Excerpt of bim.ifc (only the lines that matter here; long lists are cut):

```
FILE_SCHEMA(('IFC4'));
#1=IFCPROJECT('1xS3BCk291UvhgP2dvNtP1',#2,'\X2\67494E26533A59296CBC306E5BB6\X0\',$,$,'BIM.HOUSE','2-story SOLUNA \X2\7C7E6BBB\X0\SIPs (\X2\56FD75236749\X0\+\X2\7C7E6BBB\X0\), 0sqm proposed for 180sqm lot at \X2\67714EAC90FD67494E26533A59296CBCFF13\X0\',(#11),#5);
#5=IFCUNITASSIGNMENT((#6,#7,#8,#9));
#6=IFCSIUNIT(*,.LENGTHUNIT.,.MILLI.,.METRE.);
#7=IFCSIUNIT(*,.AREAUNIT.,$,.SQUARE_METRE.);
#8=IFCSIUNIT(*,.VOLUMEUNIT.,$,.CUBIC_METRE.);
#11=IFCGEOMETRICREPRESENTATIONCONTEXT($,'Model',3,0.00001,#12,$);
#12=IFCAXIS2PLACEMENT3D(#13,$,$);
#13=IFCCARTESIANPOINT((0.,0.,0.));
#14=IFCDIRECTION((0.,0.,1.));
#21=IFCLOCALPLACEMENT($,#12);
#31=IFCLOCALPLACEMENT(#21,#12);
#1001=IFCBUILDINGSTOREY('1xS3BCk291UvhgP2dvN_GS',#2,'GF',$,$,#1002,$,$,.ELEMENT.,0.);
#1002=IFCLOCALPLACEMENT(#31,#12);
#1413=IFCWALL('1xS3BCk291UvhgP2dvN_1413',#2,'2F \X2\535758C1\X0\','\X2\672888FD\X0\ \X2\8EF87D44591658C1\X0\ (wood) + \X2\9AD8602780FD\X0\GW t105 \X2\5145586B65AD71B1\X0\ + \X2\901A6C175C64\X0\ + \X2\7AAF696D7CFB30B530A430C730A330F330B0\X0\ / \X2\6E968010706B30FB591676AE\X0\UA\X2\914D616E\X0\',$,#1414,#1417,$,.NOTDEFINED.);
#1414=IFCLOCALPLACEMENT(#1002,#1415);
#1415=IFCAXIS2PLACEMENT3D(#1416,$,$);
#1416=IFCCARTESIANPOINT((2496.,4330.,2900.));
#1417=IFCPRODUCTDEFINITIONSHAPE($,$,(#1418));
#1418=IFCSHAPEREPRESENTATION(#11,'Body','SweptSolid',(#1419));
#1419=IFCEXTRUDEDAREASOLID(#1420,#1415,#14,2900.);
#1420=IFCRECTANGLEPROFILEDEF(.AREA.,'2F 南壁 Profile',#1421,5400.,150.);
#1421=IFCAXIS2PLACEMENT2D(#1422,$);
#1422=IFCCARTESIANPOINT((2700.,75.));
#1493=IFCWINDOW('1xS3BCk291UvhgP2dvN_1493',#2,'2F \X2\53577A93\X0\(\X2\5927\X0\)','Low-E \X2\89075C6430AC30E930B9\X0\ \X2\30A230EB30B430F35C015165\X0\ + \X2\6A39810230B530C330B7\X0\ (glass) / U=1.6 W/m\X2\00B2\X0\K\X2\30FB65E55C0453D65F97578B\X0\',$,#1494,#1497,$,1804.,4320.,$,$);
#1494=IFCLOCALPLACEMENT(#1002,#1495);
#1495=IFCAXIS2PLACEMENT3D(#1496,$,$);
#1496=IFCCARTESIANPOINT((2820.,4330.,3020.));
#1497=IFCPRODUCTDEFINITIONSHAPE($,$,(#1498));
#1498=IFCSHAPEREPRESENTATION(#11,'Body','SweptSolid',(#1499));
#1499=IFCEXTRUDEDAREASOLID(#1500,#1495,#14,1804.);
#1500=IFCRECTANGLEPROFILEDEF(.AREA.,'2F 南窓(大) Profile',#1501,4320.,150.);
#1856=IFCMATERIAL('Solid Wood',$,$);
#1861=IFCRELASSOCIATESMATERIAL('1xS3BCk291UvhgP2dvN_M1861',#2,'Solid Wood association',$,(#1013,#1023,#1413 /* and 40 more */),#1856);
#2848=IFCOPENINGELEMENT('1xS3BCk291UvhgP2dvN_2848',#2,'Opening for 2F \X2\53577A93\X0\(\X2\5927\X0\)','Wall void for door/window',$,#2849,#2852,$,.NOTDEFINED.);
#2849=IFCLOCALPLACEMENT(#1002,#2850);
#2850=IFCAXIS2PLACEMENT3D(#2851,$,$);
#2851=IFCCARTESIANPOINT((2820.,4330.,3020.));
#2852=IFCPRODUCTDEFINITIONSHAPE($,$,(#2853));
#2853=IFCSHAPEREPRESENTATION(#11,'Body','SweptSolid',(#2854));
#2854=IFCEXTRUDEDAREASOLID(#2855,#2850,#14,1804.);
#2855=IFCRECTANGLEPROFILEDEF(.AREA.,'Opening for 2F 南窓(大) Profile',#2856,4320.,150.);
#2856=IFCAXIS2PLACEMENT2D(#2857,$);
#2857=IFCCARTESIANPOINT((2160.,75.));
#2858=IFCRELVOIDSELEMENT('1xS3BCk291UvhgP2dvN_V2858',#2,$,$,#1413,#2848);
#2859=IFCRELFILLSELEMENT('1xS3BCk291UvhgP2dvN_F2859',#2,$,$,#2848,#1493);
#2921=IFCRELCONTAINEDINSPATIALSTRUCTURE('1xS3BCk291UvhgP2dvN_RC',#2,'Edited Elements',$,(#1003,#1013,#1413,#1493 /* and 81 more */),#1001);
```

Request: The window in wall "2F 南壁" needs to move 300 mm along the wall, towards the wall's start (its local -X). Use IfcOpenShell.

```python
import ifcopenshell
import ifcopenshell.api.geometry
import ifcopenshell.util.placement
import ifcopenshell.util.unit

model = ifcopenshell.open("bim.ifc")
unit_scale = ifcopenshell.util.unit.calculate_unit_scale(model)

window = model.by_guid("1xS3BCk291UvhgP2dvN_1493")
opening = window.FillsVoids[0].RelatingOpeningElement
wall = opening.VoidsElements[0].RelatingBuildingElement

wall_matrix = ifcopenshell.util.placement.get_local_placement(wall.ObjectPlacement)
shift = wall_matrix[:3, 0] * -0.3 / unit_scale
before = ifcopenshell.util.placement.get_local_placement(window.ObjectPlacement)[:3, 3].copy()

# The window is not placed relative to its opening, so move both.
for product in (opening, window):
    matrix = ifcopenshell.util.placement.get_local_placement(product.ObjectPlacement)
    matrix[:3, 3] += shift
    ifcopenshell.api.geometry.edit_object_placement(model, product=product, matrix=matrix, is_si=False)

after = ifcopenshell.util.placement.get_local_placement(window.ObjectPlacement)[:3, 3]
print("window moved by", (after - before).round(3) + 0.0)

model.write("bim_edited.ifc")
```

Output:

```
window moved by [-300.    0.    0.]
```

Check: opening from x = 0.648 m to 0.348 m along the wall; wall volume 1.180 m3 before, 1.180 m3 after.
